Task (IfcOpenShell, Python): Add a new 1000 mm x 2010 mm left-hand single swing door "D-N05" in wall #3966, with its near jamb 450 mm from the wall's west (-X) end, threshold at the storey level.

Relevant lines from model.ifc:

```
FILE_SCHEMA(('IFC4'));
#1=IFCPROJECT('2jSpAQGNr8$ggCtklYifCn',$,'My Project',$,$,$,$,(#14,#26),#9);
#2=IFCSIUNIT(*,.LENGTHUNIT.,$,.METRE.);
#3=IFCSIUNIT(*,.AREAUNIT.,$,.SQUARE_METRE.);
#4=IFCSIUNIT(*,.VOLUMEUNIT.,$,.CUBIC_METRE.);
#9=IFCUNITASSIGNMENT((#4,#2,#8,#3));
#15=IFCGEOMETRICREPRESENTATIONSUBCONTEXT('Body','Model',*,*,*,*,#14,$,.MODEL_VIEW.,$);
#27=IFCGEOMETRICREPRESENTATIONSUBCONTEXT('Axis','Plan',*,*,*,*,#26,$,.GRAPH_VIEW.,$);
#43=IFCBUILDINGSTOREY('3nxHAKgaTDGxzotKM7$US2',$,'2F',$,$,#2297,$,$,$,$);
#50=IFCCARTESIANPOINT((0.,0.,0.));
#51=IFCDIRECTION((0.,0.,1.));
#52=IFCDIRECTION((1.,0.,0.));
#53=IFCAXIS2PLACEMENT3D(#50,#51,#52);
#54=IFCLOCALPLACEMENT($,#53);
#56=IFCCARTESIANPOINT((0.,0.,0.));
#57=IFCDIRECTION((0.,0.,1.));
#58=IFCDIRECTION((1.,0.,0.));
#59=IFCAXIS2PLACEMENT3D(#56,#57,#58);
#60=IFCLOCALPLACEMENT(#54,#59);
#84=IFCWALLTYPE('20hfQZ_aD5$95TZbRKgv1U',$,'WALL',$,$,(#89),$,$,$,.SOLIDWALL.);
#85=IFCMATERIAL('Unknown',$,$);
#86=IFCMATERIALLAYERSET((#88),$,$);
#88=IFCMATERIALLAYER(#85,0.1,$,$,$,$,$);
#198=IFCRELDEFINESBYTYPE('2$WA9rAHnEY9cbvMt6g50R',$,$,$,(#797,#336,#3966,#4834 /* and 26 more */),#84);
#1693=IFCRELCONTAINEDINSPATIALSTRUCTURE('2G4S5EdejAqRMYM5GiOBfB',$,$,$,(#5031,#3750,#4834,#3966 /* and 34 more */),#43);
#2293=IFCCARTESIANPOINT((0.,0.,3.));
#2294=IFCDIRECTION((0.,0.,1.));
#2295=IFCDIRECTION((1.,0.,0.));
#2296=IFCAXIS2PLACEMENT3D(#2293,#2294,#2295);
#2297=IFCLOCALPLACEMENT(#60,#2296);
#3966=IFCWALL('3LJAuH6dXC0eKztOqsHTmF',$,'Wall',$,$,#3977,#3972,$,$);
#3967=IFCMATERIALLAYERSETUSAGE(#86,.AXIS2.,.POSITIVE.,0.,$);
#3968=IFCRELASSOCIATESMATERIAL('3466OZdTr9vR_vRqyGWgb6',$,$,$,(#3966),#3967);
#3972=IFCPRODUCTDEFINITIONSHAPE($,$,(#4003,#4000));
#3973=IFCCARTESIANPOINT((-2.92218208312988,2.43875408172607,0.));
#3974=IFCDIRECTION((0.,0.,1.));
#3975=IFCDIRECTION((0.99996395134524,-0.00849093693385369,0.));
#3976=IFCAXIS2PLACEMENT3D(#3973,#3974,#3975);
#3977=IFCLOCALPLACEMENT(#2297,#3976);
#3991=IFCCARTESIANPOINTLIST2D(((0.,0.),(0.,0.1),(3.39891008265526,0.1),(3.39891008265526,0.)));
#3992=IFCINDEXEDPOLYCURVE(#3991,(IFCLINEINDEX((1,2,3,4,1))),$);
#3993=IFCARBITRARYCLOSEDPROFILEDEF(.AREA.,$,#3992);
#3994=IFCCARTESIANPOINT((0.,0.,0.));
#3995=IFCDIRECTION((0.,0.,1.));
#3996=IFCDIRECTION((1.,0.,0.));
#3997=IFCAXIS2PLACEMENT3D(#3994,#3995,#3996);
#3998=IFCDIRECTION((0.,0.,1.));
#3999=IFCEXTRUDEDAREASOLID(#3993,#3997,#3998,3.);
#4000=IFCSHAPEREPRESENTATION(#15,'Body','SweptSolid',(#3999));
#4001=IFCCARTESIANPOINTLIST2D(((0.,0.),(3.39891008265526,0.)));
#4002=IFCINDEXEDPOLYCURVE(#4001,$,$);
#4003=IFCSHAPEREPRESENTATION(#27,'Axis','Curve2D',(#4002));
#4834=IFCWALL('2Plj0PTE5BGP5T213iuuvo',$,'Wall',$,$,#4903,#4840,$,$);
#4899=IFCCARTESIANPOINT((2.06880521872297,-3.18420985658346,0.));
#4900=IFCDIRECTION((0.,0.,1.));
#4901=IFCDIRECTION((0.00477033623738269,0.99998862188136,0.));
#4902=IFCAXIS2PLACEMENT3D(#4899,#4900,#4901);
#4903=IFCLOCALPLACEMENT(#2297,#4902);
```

```python
import numpy as np
import ifcopenshell
import ifcopenshell.api.feature
import ifcopenshell.api.geometry
import ifcopenshell.api.root
import ifcopenshell.api.spatial
import ifcopenshell.geom
import ifcopenshell.util.element
import ifcopenshell.util.placement
import ifcopenshell.util.representation
import ifcopenshell.util.shape
import ifcopenshell.util.unit

model = ifcopenshell.open("model.ifc")
unit_scale = ifcopenshell.util.unit.calculate_unit_scale(model)
settings = ifcopenshell.geom.settings()


def volume(element):
    """Net volume in cubic metres, openings subtracted."""
    shape = ifcopenshell.geom.create_shape(settings, element)
    return ifcopenshell.util.shape.get_volume(shape.geometry)


wall = model.by_guid("3LJAuH6dXC0eKztOqsHTmF")
storey = ifcopenshell.util.element.get_container(wall, ifc_class="IfcBuildingStorey")
context = ifcopenshell.util.representation.get_context(model, "Model", "Body", "MODEL_VIEW")
before = volume(wall)

width, height, from_end, sill = 1, 2.01, 0.45, 0.0  # metres

# The wall runs along its own X axis, and the end named is its -X end.
wall_shape = ifcopenshell.geom.create_shape(settings, wall)
x, y, z = ifcopenshell.util.shape.get_vertices(wall_shape.geometry).T
start = x.min() + from_end
face, thickness = float(y.min()), float(y.max() - y.min())
wall_matrix = ifcopenshell.util.placement.get_local_placement(wall.ObjectPlacement)
level = ifcopenshell.util.placement.get_local_placement(storey.ObjectPlacement)[2, 3]


def in_wall(x, y):
    """Placement at x, y metres in the wall's axes, at sill height."""
    matrix = wall_matrix.copy()
    matrix[:, 3] = wall_matrix @ np.array([x / unit_scale, y / unit_scale, 0.0, 1.0])
    matrix[2, 3] = level + sill / unit_scale
    return matrix


# Opening: a box that overshoots both wall faces by 50 mm.
opening = ifcopenshell.api.root.create_entity(model, ifc_class="IfcOpeningElement", predefined_type="OPENING")
box = ifcopenshell.api.geometry.add_wall_representation(
    model, context=context, length=width, height=height, thickness=thickness + 0.1
)
ifcopenshell.api.geometry.assign_representation(model, product=opening, representation=box)
ifcopenshell.api.geometry.edit_object_placement(model, product=opening, matrix=in_wall(start, face - 0.05), is_si=False)
ifcopenshell.api.feature.add_feature(model, feature=opening, element=wall)

door = ifcopenshell.api.root.create_entity(model, ifc_class="IfcDoor", name="D-N05", predefined_type="DOOR")
door.OverallWidth, door.OverallHeight = width / unit_scale, height / unit_scale
door.OperationType = "SINGLE_SWING_LEFT"
body = ifcopenshell.api.geometry.add_door_representation(
    model,
    context=context,
    overall_width=door.OverallWidth,
    overall_height=door.OverallHeight,
    operation_type="SINGLE_SWING_LEFT",
    lining_properties={"LiningDepth": thickness / unit_scale, "ThresholdDepth": thickness / unit_scale},
)
ifcopenshell.api.geometry.assign_representation(model, product=door, representation=body)
ifcopenshell.api.spatial.assign_container(model, products=[door], relating_structure=storey)
ifcopenshell.api.feature.add_filling(model, opening=opening, element=door)

# The lining spans the wall, so the door starts at the wall face.
ifcopenshell.api.geometry.edit_object_placement(model, product=door, matrix=in_wall(start, face), is_si=False)

after = volume(wall)

print(f"wall volume {before:.3f} -> {after:.3f} m3")

model.write("model_updated.ifc")
```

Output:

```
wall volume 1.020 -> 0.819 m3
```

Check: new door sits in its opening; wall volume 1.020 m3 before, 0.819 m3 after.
